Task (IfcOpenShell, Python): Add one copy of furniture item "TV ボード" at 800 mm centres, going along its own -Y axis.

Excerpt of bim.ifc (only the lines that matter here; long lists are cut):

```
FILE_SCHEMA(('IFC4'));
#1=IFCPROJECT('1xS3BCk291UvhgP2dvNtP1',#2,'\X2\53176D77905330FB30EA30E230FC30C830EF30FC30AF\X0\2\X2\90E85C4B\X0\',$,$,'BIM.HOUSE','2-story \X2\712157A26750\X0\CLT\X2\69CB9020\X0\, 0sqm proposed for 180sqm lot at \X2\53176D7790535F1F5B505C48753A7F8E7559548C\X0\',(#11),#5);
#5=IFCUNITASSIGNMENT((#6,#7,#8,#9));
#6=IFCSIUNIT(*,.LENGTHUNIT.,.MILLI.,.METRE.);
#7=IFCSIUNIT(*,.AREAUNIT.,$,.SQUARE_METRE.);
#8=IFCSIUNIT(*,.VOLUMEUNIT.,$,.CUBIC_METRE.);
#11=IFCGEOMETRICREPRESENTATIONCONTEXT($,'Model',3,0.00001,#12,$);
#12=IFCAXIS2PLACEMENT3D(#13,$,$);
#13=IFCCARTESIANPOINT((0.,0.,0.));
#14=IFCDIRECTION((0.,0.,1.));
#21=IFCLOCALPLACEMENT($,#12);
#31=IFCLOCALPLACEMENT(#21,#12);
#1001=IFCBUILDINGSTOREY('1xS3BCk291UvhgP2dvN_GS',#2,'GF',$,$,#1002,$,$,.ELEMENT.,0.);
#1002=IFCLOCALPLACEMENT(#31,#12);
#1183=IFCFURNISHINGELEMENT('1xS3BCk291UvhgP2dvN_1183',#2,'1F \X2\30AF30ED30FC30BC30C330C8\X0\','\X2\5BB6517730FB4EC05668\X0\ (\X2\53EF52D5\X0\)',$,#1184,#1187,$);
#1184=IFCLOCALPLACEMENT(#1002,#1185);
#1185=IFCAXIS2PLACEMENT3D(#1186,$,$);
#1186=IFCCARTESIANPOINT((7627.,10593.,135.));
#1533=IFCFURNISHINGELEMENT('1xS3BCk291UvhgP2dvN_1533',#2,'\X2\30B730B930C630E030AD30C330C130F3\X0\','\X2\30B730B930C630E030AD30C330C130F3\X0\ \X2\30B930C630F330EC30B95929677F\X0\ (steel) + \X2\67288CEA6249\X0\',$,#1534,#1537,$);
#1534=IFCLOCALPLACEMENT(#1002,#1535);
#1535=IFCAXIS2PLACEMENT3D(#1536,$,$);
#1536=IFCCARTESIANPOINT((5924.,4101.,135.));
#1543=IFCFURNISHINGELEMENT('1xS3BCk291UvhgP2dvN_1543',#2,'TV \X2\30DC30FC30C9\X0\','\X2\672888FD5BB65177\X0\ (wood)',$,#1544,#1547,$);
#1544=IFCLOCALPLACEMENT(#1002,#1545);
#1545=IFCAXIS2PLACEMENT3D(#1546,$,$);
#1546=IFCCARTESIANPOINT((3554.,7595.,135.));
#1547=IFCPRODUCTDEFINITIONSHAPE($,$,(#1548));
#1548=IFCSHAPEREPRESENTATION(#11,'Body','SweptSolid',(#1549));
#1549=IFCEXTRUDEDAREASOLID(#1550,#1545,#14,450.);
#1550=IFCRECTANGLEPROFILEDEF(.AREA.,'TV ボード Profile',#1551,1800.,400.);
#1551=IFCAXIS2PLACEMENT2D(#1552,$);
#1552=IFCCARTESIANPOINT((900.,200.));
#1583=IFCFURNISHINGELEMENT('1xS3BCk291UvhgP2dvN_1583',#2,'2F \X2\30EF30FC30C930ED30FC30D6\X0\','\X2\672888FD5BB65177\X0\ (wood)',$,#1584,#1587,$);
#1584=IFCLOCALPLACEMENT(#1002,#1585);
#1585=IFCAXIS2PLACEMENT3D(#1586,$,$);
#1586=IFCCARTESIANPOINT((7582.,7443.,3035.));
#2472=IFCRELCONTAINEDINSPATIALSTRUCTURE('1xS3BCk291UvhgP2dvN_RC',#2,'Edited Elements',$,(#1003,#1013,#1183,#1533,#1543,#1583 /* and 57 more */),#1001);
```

```python
import ifcopenshell
import ifcopenshell.api.geometry
import ifcopenshell.api.root
import ifcopenshell.util.element
import ifcopenshell.util.placement

model = ifcopenshell.open("bim.ifc")


def reuse_history(source, copy):
    """copy_class also copies each property set's owner history, people and application; keep the originals."""
    for rel in copy.IsDefinedBy:
        if rel.is_a("IfcRelDefinesByProperties") and (history := rel.RelatingPropertyDefinition.OwnerHistory):
            rel.RelatingPropertyDefinition.OwnerHistory = source.OwnerHistory
            ifcopenshell.util.element.remove_deep2(model, history)


source = model.by_guid("1xS3BCk291UvhgP2dvN_1543")
base = ifcopenshell.util.placement.get_local_placement(source.ObjectPlacement)
step = -base[:3, 1] * 800.0

for i in range(1, 2):
    copy = ifcopenshell.api.root.copy_class(model, product=source)
    copy.Representation = ifcopenshell.util.element.copy_deep(
        model, source.Representation, exclude=["IfcGeometricRepresentationContext", "IfcRepresentationMap"]
    )
    reuse_history(source, copy)
    matrix = base.copy()
    matrix[:3, 3] += i * step
    print("added at", matrix[:3, 3].round(3) + 0.0)
    ifcopenshell.api.geometry.edit_object_placement(model, product=copy, matrix=matrix, is_si=False)

model.write("bim_edited.ifc")
```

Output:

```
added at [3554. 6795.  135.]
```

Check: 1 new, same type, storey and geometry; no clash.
